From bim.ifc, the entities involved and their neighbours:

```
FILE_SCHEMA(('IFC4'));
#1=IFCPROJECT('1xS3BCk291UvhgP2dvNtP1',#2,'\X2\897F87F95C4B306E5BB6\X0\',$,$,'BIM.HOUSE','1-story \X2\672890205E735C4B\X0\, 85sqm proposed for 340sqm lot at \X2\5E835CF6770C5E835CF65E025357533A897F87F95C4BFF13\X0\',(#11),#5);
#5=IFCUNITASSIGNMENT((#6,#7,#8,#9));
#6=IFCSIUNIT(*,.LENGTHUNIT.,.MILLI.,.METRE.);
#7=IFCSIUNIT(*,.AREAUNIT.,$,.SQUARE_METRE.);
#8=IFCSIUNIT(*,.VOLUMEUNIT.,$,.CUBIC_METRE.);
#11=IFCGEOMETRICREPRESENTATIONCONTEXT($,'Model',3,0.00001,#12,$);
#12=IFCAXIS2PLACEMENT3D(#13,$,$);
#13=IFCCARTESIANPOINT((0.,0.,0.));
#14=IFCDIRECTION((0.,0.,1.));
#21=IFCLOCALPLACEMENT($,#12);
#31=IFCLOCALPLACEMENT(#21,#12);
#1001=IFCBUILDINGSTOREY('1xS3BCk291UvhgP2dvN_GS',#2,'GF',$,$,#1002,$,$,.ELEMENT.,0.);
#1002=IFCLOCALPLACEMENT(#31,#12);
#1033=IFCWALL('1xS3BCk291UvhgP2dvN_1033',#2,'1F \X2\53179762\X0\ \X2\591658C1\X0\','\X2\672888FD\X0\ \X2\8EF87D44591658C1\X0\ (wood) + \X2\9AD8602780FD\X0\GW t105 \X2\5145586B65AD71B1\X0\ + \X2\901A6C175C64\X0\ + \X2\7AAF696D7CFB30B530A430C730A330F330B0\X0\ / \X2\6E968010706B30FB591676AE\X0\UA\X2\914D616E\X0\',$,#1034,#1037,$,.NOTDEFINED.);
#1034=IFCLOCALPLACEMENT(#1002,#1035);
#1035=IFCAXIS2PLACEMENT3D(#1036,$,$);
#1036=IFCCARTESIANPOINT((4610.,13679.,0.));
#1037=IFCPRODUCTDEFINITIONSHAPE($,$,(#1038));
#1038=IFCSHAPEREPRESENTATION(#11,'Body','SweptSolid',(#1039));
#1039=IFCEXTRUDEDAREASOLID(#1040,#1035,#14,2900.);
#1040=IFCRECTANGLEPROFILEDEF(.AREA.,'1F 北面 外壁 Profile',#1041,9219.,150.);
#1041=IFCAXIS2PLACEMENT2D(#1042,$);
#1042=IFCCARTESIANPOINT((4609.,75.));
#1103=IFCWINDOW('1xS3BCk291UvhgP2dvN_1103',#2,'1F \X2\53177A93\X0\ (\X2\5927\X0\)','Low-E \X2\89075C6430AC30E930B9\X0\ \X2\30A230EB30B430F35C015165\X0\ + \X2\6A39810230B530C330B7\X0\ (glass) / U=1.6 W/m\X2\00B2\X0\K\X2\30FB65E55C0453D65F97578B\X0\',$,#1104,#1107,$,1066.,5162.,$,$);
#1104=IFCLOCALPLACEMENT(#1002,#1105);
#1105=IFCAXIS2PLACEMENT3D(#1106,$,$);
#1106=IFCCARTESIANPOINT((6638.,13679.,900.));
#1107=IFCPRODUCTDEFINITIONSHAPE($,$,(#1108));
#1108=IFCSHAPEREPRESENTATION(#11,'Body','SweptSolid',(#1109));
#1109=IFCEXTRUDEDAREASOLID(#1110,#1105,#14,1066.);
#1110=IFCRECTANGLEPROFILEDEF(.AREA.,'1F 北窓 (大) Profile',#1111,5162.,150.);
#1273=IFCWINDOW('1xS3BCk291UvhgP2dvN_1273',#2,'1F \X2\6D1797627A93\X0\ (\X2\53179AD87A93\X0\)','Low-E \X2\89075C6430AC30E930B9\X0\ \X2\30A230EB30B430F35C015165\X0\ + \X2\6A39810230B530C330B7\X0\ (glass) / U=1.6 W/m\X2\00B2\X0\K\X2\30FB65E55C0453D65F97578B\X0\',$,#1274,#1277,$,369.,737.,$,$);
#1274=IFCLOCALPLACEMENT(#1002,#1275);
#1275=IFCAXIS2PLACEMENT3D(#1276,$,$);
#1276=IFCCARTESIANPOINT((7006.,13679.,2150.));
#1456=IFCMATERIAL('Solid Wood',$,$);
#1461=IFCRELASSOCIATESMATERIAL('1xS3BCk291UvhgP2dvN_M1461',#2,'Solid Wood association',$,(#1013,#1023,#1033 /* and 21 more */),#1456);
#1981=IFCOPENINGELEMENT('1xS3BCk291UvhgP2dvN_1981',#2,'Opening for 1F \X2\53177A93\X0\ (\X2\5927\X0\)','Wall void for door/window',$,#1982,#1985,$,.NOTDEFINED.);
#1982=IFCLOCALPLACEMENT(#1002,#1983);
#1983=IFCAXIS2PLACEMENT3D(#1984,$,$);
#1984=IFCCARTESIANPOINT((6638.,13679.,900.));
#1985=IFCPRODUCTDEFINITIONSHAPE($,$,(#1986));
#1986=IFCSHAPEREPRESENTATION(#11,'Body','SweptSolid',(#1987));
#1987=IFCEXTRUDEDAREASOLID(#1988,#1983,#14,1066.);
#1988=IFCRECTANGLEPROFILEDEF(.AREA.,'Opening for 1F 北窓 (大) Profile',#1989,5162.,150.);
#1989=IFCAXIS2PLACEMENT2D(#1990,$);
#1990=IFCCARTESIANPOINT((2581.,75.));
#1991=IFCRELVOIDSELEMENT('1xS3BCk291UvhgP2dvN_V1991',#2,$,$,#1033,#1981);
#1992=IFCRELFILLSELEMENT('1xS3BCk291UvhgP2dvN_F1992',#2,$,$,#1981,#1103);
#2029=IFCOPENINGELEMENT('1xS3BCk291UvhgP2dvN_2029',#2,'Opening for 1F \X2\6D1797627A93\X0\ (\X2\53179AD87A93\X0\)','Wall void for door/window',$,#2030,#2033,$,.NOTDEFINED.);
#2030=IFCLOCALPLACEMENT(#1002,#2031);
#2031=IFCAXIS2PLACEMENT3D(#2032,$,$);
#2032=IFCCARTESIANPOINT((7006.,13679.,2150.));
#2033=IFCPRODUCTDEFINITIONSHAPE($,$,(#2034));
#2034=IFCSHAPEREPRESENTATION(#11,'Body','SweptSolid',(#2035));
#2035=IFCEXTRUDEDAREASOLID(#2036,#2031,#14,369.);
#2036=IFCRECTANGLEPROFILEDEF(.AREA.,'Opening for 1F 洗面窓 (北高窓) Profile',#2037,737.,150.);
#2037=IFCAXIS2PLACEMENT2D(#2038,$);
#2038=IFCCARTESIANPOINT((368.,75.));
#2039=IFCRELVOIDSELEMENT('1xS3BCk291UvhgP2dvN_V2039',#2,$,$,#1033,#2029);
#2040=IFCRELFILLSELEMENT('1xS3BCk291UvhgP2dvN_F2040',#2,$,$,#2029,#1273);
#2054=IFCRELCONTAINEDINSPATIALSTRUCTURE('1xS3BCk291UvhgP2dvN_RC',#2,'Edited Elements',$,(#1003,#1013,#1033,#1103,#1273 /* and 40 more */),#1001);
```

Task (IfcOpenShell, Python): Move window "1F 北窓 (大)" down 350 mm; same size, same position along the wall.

```python
import numpy as np
import ifcopenshell
import ifcopenshell.api.geometry
import ifcopenshell.util.placement
import ifcopenshell.util.unit

model = ifcopenshell.open("bim.ifc")
unit_scale = ifcopenshell.util.unit.calculate_unit_scale(model)

window = model.by_guid("1xS3BCk291UvhgP2dvN_1103")
opening = window.FillsVoids[0].RelatingOpeningElement
dz = -350.0

shift = np.array([0.0, 0.0, dz])
# The window is not placed relative to its opening, so move both.
for product in (opening, window):
    matrix = ifcopenshell.util.placement.get_local_placement(product.ObjectPlacement)
    matrix[:3, 3] += shift
    ifcopenshell.api.geometry.edit_object_placement(model, product=product, matrix=matrix, is_si=False)

print(f"moved by {dz * unit_scale:+.3f} m")

model.write("bim_edited.ifc")
```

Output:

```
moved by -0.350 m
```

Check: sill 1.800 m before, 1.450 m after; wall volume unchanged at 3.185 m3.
